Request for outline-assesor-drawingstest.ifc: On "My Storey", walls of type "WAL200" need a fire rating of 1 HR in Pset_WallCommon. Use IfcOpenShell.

First a look at what the model holds.

```python
import ifcopenshell
import ifcopenshell.util.element

model = ifcopenshell.open("outline-assesor-drawingstest.ifc")
print(model.schema)
storey = next(s for s in model.by_type("IfcBuildingStorey") if s.Name == "My Storey")
walls = [e for e in ifcopenshell.util.element.get_decomposition(storey) if e.is_a("IfcWall")]
seen = {}
for e in walls:
    element_type = ifcopenshell.util.element.get_type(e)
    key = (element_type.Name if element_type != e and element_type else None, ifcopenshell.util.element.get_pset(e, "Pset_WallCommon", "FireRating"))
    seen[key] = seen.get(key, 0) + 1
for (name, value), count in sorted(seen.items(), key=str):
    print(count, "x", name, "|", value)
```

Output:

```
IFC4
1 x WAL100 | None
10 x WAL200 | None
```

```python
import ifcopenshell
import ifcopenshell.api.pset
import ifcopenshell.util.element

model = ifcopenshell.open("outline-assesor-drawingstest.ifc")

storey = next(s for s in model.by_type("IfcBuildingStorey") if s.Name == "My Storey")
walls = [e for e in ifcopenshell.util.element.get_decomposition(storey) if e.is_a("IfcWall")]

count = 0
for e in walls:
    element_type = ifcopenshell.util.element.get_type(e)
    if element_type in (None, e) or element_type.Name != "WAL200":
        continue
    # add_pset returns the element's existing set when there is one.
    pset = ifcopenshell.api.pset.add_pset(model, product=e, name="Pset_WallCommon")
    ifcopenshell.api.pset.edit_pset(model, pset=pset, properties={"FireRating": "1 HR"})
    count += 1

print(count, "walls updated")

model.write("outline-assesor-drawingstest_edited.ifc")
```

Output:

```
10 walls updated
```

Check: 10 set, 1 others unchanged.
